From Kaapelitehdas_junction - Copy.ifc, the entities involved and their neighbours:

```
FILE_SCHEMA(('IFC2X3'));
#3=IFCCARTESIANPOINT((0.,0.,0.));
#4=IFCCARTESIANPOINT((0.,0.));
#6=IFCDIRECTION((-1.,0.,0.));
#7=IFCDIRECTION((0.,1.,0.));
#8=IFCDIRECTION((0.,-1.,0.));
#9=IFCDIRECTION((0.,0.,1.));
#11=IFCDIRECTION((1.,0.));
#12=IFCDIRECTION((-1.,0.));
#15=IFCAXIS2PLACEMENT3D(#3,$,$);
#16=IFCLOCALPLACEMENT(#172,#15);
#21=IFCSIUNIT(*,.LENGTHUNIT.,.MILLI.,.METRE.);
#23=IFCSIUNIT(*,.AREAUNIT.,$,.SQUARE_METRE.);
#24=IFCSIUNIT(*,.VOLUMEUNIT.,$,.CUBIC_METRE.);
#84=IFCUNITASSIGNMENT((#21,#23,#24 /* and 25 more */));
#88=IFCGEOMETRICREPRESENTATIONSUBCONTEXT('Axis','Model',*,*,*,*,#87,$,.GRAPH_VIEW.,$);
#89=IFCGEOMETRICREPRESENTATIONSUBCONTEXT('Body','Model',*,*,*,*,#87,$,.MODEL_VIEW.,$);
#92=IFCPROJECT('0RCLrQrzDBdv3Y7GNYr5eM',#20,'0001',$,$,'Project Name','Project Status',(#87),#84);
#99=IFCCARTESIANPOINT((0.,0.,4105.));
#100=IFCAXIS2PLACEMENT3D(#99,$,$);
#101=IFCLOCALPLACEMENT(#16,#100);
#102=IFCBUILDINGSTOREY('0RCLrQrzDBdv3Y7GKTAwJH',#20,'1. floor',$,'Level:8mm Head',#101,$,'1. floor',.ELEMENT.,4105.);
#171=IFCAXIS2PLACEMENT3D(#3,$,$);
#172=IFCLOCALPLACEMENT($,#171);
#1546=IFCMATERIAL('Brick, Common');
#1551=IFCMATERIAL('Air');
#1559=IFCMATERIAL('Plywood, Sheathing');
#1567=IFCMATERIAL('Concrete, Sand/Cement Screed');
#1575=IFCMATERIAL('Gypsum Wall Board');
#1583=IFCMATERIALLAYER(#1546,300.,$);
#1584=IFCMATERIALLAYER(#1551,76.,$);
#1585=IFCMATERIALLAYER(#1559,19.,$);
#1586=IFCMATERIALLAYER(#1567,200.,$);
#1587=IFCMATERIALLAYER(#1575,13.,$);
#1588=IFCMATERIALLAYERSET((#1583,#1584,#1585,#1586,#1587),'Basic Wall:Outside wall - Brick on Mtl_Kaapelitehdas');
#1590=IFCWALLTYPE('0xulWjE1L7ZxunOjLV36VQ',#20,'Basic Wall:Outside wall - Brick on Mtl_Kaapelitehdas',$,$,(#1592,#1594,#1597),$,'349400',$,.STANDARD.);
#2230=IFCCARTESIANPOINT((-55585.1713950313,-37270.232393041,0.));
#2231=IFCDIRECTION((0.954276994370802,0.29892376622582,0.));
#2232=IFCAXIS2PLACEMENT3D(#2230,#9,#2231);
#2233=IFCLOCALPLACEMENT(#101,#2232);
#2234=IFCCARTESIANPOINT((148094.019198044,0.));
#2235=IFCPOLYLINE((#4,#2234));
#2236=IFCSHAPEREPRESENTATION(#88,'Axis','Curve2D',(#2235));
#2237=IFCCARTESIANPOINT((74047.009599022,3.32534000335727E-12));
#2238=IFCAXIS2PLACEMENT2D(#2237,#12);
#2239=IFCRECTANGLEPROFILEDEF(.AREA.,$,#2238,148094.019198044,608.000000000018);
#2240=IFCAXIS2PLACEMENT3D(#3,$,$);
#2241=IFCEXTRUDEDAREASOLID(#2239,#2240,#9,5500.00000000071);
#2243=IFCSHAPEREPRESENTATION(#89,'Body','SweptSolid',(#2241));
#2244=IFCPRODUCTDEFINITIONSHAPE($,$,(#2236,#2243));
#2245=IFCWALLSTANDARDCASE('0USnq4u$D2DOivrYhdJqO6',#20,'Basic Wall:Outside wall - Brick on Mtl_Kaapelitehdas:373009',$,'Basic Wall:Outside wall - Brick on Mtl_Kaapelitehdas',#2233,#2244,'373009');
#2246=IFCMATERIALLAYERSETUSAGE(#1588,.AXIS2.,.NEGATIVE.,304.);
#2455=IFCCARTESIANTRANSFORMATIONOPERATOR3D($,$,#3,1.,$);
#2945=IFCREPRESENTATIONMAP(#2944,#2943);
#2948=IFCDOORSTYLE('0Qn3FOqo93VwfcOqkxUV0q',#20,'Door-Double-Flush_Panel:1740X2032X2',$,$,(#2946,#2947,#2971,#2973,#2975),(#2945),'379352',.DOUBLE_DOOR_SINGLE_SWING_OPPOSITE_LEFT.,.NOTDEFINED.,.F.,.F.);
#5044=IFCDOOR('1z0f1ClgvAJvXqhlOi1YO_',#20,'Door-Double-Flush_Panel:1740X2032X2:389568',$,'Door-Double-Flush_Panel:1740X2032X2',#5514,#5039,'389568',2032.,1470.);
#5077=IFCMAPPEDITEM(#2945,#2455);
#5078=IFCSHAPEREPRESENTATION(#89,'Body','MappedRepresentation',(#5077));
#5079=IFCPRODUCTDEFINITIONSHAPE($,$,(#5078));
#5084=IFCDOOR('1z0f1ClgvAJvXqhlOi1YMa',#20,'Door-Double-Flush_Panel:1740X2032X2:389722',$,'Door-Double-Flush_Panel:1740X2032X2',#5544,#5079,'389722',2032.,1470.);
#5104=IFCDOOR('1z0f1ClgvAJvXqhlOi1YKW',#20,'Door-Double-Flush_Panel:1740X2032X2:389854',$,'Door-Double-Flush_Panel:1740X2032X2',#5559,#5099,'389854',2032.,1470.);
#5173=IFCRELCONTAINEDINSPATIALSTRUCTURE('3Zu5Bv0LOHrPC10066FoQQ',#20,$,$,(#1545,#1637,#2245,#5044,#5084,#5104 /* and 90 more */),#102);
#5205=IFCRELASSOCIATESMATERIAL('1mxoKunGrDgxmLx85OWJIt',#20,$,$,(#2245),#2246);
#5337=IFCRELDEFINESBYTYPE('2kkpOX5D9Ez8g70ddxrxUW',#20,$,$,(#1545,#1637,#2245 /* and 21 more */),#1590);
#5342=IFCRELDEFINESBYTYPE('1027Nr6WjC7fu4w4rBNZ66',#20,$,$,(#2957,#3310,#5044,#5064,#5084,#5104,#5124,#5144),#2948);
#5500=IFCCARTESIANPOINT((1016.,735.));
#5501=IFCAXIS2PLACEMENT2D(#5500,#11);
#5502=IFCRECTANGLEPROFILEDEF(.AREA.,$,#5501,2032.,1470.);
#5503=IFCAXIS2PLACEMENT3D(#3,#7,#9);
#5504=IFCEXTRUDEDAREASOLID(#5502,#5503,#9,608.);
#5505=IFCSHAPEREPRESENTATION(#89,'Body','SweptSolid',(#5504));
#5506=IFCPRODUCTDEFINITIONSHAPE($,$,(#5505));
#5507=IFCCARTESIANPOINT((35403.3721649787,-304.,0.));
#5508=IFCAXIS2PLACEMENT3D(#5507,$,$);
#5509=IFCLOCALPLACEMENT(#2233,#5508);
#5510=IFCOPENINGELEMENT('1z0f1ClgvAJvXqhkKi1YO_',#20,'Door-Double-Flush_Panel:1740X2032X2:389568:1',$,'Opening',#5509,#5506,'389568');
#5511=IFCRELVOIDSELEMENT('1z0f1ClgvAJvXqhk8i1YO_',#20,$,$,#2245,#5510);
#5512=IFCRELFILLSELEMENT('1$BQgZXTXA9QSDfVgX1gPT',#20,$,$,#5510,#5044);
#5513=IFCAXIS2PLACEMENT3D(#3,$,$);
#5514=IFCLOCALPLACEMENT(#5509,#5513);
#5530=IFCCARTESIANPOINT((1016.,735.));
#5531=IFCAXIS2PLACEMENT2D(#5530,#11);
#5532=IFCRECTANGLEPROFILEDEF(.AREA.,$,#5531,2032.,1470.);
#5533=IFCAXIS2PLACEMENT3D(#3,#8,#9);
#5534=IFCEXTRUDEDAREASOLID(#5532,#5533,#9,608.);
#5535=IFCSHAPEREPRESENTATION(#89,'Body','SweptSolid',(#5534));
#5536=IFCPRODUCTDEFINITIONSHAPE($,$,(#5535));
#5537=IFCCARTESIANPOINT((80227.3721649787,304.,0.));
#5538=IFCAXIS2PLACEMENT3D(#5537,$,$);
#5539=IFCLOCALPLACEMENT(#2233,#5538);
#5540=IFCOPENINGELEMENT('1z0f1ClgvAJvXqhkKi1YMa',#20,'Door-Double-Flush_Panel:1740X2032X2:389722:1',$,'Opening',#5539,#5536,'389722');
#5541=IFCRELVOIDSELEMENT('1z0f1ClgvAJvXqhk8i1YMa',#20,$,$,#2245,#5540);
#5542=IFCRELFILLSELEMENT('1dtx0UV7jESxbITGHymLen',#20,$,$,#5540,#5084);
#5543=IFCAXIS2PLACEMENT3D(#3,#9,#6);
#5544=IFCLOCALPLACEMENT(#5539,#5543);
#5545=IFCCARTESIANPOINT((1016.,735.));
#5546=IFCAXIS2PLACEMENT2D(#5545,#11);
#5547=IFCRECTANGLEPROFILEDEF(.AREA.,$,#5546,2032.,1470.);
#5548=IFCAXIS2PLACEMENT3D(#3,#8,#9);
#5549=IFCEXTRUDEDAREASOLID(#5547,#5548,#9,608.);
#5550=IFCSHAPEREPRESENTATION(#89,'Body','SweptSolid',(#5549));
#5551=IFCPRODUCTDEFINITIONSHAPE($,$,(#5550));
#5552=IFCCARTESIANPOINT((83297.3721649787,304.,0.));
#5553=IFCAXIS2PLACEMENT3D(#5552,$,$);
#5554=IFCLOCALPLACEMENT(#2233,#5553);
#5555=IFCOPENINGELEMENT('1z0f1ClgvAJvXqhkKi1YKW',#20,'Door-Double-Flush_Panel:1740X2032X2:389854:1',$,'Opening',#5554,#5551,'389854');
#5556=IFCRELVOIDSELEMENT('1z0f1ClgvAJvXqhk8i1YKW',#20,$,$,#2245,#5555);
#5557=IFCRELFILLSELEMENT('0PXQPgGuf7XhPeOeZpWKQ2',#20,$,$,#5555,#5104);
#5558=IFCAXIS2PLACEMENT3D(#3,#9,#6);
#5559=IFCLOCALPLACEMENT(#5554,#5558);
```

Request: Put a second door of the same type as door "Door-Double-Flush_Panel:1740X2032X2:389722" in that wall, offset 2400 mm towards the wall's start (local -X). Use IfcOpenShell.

```python
import ifcopenshell
import ifcopenshell.api.feature
import ifcopenshell.api.geometry
import ifcopenshell.api.root
import ifcopenshell.geom
import ifcopenshell.util.element
import ifcopenshell.util.placement
import ifcopenshell.util.shape
import ifcopenshell.util.unit

model = ifcopenshell.open("Kaapelitehdas_junction - Copy.ifc")
unit_scale = ifcopenshell.util.unit.calculate_unit_scale(model)
settings = ifcopenshell.geom.settings()


def volume(element):
    """Net volume in cubic metres, openings subtracted."""
    shape = ifcopenshell.geom.create_shape(settings, element)
    return ifcopenshell.util.shape.get_volume(shape.geometry)


def reuse_history(source, copy):
    """copy_class also copies each property set's owner history, people and application; keep the originals."""
    for rel in copy.IsDefinedBy:
        if rel.is_a("IfcRelDefinesByProperties") and (history := rel.RelatingPropertyDefinition.OwnerHistory):
            rel.RelatingPropertyDefinition.OwnerHistory = source.OwnerHistory
            ifcopenshell.util.element.remove_deep2(model, history)


door = model.by_guid("1z0f1ClgvAJvXqhlOi1YMa")
opening = door.FillsVoids[0].RelatingOpeningElement
wall = opening.VoidsElements[0].RelatingBuildingElement
before = volume(wall)
shift = ifcopenshell.util.placement.get_local_placement(wall.ObjectPlacement)[:3, 0] * -2.4 / unit_scale

# copy_class copies the void relationship, type, container and properties, but no geometry.
new_opening = ifcopenshell.api.root.copy_class(model, product=opening)
new_opening.Representation = ifcopenshell.util.element.copy_deep(
    model, opening.Representation, exclude=["IfcGeometricRepresentationContext", "IfcRepresentationMap"]
)
new_opening.Name = "Door-Double-Flush_Panel:1740X2032X2"
new_opening.Tag = None
new_door = ifcopenshell.api.root.copy_class(model, product=door)
new_door.Representation = ifcopenshell.util.element.copy_deep(
    model, door.Representation, exclude=["IfcGeometricRepresentationContext", "IfcRepresentationMap"]
)
new_door.Name = "Door-Double-Flush_Panel:1740X2032X2"
new_door.Tag = None
reuse_history(door, new_door)
fills = ifcopenshell.api.feature.add_filling(model, opening=new_opening, element=new_door)
fills.OwnerHistory = new_door.OwnerHistory  # required in IFC2X3

for old, new in ((opening, new_opening), (door, new_door)):
    matrix = ifcopenshell.util.placement.get_local_placement(old.ObjectPlacement)
    matrix[:3, 3] += shift
    ifcopenshell.api.geometry.edit_object_placement(model, product=new, matrix=matrix, is_si=False)

after = volume(wall)

print(f"wall volume {before:.3f} -> {after:.3f} m3")

model.write("Kaapelitehdas_junction - Copy-out.ifc")
```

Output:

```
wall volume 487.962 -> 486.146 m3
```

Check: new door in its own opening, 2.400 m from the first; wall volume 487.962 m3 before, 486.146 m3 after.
